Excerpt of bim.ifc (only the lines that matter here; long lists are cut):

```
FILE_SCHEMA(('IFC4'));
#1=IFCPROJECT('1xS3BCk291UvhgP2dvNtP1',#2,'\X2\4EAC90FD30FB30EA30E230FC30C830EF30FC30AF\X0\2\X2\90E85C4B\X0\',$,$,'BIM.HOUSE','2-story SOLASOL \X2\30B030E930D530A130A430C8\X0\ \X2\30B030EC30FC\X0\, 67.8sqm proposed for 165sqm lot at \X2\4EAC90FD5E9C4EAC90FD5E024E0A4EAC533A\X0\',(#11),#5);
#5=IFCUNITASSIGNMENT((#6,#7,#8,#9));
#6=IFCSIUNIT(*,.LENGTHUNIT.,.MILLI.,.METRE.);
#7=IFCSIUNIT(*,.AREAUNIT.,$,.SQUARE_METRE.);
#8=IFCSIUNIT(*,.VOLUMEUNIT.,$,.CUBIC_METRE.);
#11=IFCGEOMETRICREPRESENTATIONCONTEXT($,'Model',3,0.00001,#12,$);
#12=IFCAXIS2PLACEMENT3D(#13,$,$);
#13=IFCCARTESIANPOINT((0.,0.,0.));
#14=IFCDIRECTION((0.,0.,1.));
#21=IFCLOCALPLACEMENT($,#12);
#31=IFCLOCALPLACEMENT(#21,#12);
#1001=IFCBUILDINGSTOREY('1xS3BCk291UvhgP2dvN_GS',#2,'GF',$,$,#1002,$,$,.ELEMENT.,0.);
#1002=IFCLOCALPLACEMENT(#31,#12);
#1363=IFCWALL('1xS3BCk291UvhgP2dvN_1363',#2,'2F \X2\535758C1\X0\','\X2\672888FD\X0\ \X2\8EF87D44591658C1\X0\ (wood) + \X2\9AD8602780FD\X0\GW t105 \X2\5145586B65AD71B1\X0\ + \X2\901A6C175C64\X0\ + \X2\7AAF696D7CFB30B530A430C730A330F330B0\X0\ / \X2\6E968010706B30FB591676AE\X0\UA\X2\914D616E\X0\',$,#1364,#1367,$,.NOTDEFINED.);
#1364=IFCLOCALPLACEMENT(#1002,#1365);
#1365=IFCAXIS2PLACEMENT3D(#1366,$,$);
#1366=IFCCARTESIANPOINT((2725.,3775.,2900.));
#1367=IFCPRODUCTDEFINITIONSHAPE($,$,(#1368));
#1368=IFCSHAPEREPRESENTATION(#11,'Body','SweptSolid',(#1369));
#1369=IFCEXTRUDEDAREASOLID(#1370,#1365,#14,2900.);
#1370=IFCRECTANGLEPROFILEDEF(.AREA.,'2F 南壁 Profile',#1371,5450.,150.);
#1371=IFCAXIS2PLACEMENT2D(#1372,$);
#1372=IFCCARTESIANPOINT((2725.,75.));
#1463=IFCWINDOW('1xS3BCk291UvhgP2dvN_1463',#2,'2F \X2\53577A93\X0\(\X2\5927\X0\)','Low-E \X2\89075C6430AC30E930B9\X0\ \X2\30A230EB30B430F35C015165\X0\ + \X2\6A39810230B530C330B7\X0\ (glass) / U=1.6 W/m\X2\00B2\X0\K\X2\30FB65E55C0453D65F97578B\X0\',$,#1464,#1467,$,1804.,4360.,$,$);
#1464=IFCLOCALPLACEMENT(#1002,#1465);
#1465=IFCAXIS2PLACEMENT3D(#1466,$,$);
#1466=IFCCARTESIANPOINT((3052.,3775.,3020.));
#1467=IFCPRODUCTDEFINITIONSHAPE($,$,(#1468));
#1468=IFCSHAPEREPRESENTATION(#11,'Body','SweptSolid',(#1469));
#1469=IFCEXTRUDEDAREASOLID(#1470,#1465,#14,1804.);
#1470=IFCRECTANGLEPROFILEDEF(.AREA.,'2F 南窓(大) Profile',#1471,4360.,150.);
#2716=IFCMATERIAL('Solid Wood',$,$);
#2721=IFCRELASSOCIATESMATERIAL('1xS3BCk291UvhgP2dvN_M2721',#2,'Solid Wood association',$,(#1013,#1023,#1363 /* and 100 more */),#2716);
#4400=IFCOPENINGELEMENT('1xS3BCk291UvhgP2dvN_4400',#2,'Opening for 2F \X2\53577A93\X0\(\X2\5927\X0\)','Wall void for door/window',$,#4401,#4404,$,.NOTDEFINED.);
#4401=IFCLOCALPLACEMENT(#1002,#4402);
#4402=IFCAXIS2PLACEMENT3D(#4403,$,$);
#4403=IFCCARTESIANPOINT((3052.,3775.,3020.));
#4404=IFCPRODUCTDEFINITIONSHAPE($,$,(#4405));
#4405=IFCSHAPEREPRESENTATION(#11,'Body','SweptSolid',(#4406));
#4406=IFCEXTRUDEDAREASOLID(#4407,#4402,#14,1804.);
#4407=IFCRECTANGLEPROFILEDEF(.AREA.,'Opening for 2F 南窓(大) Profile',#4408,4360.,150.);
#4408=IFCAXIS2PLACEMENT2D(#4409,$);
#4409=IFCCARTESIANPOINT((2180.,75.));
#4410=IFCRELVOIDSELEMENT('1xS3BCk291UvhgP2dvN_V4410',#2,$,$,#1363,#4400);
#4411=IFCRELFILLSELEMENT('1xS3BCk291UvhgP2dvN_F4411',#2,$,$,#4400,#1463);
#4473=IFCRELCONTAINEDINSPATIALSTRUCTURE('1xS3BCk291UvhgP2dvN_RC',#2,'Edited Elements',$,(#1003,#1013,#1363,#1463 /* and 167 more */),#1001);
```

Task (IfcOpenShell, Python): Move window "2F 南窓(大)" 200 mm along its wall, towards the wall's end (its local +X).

```python
import ifcopenshell
import ifcopenshell.api.geometry
import ifcopenshell.util.placement

model = ifcopenshell.open("bim.ifc")

window = model.by_guid("1xS3BCk291UvhgP2dvN_1463")
opening = window.FillsVoids[0].RelatingOpeningElement
wall = opening.VoidsElements[0].RelatingBuildingElement

wall_matrix = ifcopenshell.util.placement.get_local_placement(wall.ObjectPlacement)
shift = wall_matrix[:3, 0] * 200.0
before = ifcopenshell.util.placement.get_local_placement(window.ObjectPlacement)[:3, 3].copy()

# The window is not placed relative to its opening, so move both.
for product in (opening, window):
    matrix = ifcopenshell.util.placement.get_local_placement(product.ObjectPlacement)
    matrix[:3, 3] += shift
    ifcopenshell.api.geometry.edit_object_placement(model, product=product, matrix=matrix, is_si=False)

after = ifcopenshell.util.placement.get_local_placement(window.ObjectPlacement)[:3, 3]
print("window moved by", (after - before).round(3) + 0.0)

model.write("bim_v2.ifc")
```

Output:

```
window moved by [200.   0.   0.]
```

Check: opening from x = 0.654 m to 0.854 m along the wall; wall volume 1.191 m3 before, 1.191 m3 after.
